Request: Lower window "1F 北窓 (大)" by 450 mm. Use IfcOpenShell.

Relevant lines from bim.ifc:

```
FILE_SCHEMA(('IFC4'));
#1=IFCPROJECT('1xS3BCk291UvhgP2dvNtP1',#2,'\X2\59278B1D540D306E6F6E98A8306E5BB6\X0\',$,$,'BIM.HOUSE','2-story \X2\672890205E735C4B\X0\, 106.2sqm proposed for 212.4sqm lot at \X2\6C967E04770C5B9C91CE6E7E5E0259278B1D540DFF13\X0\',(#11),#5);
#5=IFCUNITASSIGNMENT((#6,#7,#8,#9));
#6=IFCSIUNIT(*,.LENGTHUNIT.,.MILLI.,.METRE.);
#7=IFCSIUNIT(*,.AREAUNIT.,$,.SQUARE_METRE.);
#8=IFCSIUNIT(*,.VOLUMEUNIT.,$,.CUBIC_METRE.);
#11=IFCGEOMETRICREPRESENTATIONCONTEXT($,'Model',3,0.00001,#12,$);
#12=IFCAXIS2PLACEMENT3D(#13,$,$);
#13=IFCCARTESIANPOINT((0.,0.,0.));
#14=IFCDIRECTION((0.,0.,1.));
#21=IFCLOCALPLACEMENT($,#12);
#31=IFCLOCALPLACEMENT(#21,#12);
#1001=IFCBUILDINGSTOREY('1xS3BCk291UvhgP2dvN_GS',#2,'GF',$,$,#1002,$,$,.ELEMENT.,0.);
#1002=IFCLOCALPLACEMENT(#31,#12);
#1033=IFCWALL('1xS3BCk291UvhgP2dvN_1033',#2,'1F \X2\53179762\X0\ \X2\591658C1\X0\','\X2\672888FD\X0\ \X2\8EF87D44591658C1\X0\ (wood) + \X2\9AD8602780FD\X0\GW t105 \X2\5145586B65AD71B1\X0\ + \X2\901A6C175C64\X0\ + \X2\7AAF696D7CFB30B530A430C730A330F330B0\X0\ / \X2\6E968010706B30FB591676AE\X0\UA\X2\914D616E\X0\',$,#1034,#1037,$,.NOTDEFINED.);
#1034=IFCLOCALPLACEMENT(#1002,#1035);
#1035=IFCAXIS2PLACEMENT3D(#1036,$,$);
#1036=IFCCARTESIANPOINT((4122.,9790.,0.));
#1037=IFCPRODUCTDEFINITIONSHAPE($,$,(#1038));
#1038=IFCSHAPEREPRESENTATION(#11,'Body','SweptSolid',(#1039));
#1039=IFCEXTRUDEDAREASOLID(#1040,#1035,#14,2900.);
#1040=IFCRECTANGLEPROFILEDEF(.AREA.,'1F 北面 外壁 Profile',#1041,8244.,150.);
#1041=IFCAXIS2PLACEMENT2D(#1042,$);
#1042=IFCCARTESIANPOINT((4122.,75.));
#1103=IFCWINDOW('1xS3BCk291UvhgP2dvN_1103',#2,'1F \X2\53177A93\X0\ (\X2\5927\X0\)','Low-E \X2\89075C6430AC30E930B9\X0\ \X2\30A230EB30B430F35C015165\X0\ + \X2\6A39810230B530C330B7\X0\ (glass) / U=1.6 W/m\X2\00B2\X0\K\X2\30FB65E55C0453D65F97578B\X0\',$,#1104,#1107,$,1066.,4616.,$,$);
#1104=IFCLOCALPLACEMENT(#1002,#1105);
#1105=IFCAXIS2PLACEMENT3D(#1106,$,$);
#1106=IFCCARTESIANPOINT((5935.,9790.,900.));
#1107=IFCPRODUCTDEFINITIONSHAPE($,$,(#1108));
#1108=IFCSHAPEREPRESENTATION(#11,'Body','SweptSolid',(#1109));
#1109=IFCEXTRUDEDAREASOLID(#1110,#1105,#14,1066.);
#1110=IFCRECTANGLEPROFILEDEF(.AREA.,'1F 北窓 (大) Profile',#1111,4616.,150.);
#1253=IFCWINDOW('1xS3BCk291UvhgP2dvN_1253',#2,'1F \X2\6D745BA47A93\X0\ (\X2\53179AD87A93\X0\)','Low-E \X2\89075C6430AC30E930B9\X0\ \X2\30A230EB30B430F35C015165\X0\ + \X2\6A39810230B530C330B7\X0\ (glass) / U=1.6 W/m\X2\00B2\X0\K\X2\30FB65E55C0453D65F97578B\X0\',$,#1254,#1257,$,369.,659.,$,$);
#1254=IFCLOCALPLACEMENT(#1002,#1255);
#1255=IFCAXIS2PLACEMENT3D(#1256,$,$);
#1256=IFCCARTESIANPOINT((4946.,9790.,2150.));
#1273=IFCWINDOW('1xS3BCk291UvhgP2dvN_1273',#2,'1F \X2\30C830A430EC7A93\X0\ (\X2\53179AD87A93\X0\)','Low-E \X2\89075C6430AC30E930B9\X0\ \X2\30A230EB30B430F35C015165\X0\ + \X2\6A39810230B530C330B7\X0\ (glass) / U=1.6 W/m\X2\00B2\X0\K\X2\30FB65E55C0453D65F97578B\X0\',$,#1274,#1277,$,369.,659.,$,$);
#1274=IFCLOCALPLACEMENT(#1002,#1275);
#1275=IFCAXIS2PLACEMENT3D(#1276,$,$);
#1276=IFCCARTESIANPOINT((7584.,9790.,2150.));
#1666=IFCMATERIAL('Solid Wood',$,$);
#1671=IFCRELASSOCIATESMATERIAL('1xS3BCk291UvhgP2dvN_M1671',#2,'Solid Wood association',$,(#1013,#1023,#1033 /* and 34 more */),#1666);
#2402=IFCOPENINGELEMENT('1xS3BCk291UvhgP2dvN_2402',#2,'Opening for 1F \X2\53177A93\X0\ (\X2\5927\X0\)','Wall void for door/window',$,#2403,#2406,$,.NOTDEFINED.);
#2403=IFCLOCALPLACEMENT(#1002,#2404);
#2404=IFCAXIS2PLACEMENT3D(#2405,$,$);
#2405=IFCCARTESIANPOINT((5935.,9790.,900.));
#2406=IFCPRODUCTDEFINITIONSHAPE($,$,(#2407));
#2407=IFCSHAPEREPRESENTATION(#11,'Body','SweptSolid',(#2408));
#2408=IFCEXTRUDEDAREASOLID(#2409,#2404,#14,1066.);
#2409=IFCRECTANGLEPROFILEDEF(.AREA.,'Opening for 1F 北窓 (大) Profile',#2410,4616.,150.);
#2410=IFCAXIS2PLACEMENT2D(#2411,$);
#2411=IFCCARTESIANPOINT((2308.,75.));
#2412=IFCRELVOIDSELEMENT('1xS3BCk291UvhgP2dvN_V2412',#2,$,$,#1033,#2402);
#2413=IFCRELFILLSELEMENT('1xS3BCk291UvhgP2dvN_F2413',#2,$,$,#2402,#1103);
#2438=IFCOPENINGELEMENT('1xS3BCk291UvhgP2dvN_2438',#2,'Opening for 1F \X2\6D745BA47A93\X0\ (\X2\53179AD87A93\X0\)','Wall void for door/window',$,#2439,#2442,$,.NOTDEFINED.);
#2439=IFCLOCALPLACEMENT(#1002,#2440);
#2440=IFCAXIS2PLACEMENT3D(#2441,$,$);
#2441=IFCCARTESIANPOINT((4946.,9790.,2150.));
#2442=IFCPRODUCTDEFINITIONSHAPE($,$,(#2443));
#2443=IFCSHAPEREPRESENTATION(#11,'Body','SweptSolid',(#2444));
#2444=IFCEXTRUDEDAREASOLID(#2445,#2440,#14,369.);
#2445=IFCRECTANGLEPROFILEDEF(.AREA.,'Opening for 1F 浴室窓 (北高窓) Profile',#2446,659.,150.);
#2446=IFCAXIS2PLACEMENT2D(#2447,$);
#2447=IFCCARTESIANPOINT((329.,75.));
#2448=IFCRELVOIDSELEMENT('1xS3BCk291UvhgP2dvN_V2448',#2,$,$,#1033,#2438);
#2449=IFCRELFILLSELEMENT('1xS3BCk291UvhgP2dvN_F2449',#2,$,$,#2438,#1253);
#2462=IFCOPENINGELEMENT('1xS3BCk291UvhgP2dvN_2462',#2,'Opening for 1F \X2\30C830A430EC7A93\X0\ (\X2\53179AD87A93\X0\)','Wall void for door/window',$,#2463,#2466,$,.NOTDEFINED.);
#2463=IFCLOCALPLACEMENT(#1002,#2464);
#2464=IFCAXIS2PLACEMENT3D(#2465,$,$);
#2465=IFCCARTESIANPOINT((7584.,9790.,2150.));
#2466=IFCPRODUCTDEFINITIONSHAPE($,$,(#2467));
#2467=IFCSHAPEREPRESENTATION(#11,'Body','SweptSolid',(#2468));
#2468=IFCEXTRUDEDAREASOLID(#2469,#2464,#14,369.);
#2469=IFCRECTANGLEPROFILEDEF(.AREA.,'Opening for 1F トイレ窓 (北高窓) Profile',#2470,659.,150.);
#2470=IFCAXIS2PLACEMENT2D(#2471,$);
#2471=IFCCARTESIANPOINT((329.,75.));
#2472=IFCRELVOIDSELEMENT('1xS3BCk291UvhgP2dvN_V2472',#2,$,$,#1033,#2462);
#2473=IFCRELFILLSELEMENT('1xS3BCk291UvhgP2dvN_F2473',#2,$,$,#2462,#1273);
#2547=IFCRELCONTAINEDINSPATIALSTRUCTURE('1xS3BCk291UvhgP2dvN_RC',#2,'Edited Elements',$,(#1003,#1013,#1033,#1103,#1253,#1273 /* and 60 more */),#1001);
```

```python
import numpy as np
import ifcopenshell
import ifcopenshell.api.geometry
import ifcopenshell.util.placement
import ifcopenshell.util.unit

model = ifcopenshell.open("bim.ifc")
unit_scale = ifcopenshell.util.unit.calculate_unit_scale(model)

window = model.by_id(1103)
opening = window.FillsVoids[0].RelatingOpeningElement
dz = -0.45 / unit_scale

shift = np.array([0.0, 0.0, dz])
# The window is not placed relative to its opening, so move both.
for product in (opening, window):
    matrix = ifcopenshell.util.placement.get_local_placement(product.ObjectPlacement)
    matrix[:3, 3] += shift
    ifcopenshell.api.geometry.edit_object_placement(model, product=product, matrix=matrix, is_si=False)

print(f"moved by {dz * unit_scale:+.3f} m")

model.write("bim_rev.ifc")
```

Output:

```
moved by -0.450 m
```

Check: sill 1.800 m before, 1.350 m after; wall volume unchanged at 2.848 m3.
